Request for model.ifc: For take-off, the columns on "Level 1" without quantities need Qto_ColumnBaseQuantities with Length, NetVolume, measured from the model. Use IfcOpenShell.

First a look at what the model holds.

```python
import ifcopenshell
import ifcopenshell.util.element
import ifcopenshell.util.unit

model = ifcopenshell.open("model.ifc")
print(model.schema)
for unit_type in ("LENGTHUNIT", "AREAUNIT", "VOLUMEUNIT"):
    print(unit_type, ifcopenshell.util.unit.calculate_unit_scale(model, unit_type))
storey = next(s for s in model.by_type("IfcBuildingStorey") if s.Name == "Level 1")
columns = [e for e in ifcopenshell.util.element.get_decomposition(storey) if e.is_a("IfcColumn")]
for e in sorted(columns, key=lambda e: e.id()):
    print(e.id(), e.is_a(), e.Name, list(ifcopenshell.util.element.get_psets(e, qtos_only=True)), sep=" | ")
```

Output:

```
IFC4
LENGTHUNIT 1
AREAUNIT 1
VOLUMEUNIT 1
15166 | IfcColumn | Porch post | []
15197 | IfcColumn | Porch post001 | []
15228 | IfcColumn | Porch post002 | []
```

```python
import ifcopenshell
import ifcopenshell.api.pset
import ifcopenshell.geom
import ifcopenshell.util.element
import ifcopenshell.util.shape
import ifcopenshell.util.unit

model = ifcopenshell.open("model.ifc")
unit_scale = ifcopenshell.util.unit.calculate_unit_scale(model)
volume_scale = ifcopenshell.util.unit.calculate_unit_scale(model, "VOLUMEUNIT")
settings = ifcopenshell.geom.settings()

storey = next(s for s in model.by_type("IfcBuildingStorey") if s.Name == "Level 1")
columns = [e for e in ifcopenshell.util.element.get_decomposition(storey) if e.is_a("IfcColumn")]

for e in sorted(columns, key=lambda e: e.id()):
    if ifcopenshell.util.element.get_psets(e, qtos_only=True, should_inherit=False):
        continue
    # Geometry comes back in metres, in the element's own axes.
    shape = ifcopenshell.geom.create_shape(settings, e)
    values = {
        "Length": ifcopenshell.util.shape.get_z(shape.geometry) / unit_scale,
        "NetVolume": ifcopenshell.util.shape.get_volume(shape.geometry) / volume_scale,
    }
    qto = ifcopenshell.api.pset.add_qto(model, product=e, name="Qto_ColumnBaseQuantities")
    ifcopenshell.api.pset.edit_qto(model, qto=qto, properties=values)
    print(e.id(), {k: round(v, 3) for k, v in values.items()})

model.write("model_edited.ifc")
```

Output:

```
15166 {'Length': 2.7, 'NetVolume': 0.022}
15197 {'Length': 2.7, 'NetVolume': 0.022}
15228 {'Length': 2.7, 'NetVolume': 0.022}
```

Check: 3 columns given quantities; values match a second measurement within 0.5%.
